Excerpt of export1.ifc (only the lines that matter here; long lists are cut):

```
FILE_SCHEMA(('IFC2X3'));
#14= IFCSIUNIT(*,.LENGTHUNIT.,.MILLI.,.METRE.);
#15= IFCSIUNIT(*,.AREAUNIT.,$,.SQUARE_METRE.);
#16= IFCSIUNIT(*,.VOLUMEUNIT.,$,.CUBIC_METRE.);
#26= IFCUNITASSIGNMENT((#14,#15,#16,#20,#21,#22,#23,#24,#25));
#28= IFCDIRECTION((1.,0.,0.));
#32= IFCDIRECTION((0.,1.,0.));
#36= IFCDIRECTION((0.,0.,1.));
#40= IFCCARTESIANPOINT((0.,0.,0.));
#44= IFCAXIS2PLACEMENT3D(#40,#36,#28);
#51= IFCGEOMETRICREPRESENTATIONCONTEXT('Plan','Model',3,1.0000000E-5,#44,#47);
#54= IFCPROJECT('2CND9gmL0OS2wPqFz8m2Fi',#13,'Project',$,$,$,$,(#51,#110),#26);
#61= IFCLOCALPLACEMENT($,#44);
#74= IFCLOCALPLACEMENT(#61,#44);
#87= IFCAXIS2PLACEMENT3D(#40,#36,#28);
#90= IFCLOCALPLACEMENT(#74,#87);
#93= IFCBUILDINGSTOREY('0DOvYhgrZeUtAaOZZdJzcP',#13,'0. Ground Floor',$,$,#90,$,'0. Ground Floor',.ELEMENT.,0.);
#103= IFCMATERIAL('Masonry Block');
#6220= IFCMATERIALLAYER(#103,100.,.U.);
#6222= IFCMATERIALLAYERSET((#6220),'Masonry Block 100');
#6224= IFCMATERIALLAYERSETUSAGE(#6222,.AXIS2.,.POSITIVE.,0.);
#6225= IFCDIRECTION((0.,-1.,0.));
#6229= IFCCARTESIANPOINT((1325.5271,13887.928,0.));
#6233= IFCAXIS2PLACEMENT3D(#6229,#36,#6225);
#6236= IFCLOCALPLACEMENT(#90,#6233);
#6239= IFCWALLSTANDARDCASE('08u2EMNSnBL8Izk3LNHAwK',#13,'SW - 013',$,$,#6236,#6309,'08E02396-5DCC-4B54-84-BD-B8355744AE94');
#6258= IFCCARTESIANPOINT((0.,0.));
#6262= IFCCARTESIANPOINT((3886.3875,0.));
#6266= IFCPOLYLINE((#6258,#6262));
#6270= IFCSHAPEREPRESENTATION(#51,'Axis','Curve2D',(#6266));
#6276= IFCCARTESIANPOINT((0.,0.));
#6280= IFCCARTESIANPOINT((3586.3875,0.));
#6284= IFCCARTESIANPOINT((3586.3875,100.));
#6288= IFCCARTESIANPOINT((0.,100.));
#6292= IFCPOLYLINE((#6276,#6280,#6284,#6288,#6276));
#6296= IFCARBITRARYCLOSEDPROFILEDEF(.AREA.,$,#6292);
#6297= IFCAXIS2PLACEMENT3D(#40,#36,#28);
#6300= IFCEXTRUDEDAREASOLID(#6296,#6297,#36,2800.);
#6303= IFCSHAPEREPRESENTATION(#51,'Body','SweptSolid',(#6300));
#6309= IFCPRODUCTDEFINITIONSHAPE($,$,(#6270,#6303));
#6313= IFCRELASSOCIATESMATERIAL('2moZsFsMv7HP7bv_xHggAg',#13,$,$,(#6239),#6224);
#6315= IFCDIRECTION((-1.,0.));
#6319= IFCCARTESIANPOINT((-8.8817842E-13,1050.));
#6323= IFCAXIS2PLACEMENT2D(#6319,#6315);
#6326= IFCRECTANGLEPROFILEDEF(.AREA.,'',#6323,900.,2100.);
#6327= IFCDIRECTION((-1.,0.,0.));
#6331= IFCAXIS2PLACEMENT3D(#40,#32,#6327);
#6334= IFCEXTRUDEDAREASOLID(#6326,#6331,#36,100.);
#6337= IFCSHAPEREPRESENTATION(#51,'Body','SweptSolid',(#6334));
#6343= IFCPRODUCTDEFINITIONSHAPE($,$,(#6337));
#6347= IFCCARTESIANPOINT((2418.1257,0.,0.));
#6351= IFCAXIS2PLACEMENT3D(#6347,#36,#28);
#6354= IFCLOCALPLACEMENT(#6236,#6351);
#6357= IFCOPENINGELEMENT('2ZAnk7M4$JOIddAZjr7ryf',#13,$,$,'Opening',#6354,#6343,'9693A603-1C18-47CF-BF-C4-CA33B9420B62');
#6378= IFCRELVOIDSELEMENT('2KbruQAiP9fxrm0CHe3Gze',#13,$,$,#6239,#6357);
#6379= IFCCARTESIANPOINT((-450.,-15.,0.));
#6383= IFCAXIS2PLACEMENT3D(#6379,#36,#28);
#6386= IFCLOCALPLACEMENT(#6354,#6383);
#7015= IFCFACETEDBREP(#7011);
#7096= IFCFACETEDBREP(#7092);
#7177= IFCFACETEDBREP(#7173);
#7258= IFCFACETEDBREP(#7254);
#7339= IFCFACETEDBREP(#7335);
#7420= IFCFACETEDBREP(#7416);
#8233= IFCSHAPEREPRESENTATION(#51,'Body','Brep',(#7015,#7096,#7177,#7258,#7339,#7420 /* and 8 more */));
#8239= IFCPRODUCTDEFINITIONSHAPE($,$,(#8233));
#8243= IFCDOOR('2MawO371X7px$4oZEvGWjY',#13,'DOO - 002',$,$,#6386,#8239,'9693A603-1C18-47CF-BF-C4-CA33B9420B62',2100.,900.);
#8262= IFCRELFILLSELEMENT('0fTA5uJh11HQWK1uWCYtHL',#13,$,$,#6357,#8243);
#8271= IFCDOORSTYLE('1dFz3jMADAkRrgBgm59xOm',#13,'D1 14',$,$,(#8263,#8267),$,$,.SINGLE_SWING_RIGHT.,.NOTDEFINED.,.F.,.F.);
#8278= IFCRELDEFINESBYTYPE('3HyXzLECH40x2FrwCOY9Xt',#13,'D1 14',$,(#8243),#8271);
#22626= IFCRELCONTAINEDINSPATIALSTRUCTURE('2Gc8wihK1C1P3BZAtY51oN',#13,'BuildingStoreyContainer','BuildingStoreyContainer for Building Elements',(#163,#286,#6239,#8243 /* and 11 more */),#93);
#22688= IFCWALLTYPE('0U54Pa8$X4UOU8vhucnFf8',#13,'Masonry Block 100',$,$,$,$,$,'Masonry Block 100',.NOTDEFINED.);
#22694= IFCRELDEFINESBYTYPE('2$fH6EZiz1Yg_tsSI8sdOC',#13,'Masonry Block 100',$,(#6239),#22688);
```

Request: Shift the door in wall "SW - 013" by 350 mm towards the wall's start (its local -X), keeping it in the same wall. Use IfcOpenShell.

```python
import ifcopenshell
import ifcopenshell.api.geometry
import ifcopenshell.util.placement
import ifcopenshell.util.unit

model = ifcopenshell.open("export1.ifc")
unit_scale = ifcopenshell.util.unit.calculate_unit_scale(model)

door = model.by_guid("2MawO371X7px$4oZEvGWjY")
opening = door.FillsVoids[0].RelatingOpeningElement
wall = opening.VoidsElements[0].RelatingBuildingElement

wall_matrix = ifcopenshell.util.placement.get_local_placement(wall.ObjectPlacement)
shift = wall_matrix[:3, 0] * -0.35 / unit_scale
before = ifcopenshell.util.placement.get_local_placement(door.ObjectPlacement)[:3, 3].copy()

# The door is placed relative to its opening, so it follows when the opening moves.
matrix = ifcopenshell.util.placement.get_local_placement(opening.ObjectPlacement)
matrix[:3, 3] += shift
ifcopenshell.api.geometry.edit_object_placement(
    model, product=opening, matrix=matrix, is_si=False, should_transform_children=True
)

after = ifcopenshell.util.placement.get_local_placement(door.ObjectPlacement)[:3, 3]
print("door moved by", (after - before).round(3) + 0.0)

model.write("export1_v2.ifc")
```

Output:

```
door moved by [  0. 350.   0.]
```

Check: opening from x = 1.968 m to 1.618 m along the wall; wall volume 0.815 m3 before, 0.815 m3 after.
